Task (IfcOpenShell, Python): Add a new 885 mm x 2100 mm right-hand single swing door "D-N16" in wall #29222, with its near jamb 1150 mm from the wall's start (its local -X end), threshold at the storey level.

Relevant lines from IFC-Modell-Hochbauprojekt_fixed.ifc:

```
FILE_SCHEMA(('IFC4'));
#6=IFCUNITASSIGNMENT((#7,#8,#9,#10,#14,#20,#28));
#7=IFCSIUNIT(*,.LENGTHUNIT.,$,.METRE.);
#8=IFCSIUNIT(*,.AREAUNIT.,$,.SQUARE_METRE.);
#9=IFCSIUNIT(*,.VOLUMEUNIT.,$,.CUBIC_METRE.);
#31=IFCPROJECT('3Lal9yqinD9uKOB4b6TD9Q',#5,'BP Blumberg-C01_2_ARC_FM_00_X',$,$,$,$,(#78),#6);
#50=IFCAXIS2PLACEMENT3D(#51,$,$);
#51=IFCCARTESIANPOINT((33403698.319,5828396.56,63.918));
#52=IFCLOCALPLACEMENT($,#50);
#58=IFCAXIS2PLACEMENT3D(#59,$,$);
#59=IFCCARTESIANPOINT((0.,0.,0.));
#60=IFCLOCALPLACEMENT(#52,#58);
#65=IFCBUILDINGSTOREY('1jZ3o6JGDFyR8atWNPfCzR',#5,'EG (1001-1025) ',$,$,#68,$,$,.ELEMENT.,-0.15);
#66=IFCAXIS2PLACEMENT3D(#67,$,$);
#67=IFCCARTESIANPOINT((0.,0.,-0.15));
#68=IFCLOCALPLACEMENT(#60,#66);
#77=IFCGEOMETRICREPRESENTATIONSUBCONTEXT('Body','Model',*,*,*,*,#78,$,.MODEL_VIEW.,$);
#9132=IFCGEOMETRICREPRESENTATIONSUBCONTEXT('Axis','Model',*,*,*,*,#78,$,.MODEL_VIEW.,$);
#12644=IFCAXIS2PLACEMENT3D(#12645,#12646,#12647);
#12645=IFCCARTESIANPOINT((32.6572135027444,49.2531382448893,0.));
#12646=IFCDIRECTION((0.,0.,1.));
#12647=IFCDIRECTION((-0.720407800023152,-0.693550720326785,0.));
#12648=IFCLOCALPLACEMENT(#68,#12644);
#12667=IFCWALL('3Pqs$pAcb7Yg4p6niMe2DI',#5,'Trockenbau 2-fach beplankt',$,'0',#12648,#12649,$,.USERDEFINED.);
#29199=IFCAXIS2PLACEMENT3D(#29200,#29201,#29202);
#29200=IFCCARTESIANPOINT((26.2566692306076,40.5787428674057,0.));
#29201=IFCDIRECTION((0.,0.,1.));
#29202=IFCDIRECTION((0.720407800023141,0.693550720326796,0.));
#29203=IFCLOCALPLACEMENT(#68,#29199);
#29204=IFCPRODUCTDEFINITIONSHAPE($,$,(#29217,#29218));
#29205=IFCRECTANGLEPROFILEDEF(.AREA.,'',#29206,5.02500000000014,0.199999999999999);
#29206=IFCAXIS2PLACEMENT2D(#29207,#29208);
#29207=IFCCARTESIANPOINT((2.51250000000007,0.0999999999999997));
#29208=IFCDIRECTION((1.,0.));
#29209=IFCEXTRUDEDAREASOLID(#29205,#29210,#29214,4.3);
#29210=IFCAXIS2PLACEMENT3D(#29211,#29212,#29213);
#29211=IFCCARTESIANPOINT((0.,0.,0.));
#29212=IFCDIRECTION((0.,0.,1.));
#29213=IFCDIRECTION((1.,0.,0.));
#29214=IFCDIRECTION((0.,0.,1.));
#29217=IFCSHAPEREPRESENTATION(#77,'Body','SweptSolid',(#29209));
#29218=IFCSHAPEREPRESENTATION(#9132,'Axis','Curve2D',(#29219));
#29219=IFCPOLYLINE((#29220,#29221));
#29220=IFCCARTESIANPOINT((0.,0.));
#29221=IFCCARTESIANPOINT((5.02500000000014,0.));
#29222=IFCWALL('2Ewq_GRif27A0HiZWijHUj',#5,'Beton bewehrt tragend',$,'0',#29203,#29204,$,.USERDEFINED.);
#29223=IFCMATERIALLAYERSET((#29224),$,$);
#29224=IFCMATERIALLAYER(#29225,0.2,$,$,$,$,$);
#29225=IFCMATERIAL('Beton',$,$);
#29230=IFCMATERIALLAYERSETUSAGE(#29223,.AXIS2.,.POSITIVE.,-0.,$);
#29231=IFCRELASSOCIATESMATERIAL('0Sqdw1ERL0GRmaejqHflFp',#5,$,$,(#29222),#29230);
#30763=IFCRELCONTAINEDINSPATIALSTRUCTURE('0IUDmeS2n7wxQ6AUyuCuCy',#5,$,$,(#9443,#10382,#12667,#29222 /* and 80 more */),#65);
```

```python
import numpy as np
import ifcopenshell
import ifcopenshell.api.feature
import ifcopenshell.api.geometry
import ifcopenshell.api.root
import ifcopenshell.api.spatial
import ifcopenshell.geom
import ifcopenshell.util.element
import ifcopenshell.util.placement
import ifcopenshell.util.representation
import ifcopenshell.util.shape
import ifcopenshell.util.unit

model = ifcopenshell.open("IFC-Modell-Hochbauprojekt_fixed.ifc")
unit_scale = ifcopenshell.util.unit.calculate_unit_scale(model)
settings = ifcopenshell.geom.settings()


def volume(element):
    """Net volume in cubic metres, openings subtracted."""
    shape = ifcopenshell.geom.create_shape(settings, element)
    return ifcopenshell.util.shape.get_volume(shape.geometry)


wall = model.by_id(29222)
storey = ifcopenshell.util.element.get_container(wall, ifc_class="IfcBuildingStorey")
context = ifcopenshell.util.representation.get_context(model, "Model", "Body", "MODEL_VIEW")
before = volume(wall)

width, height, from_end, sill = 0.885, 2.1, 1.15, 0.0  # metres

# The wall runs along its own X axis, and the end named is its -X end.
wall_shape = ifcopenshell.geom.create_shape(settings, wall)
x, y, z = ifcopenshell.util.shape.get_vertices(wall_shape.geometry).T
start = x.min() + from_end
face, thickness = float(y.min()), float(y.max() - y.min())
wall_matrix = ifcopenshell.util.placement.get_local_placement(wall.ObjectPlacement)
level = ifcopenshell.util.placement.get_local_placement(storey.ObjectPlacement)[2, 3]


def in_wall(x, y):
    """Placement at x, y metres in the wall's axes, at sill height."""
    matrix = wall_matrix.copy()
    matrix[:, 3] = wall_matrix @ np.array([x / unit_scale, y / unit_scale, 0.0, 1.0])
    matrix[2, 3] = level + sill / unit_scale
    return matrix


# Opening: a box that overshoots both wall faces by 50 mm.
opening = ifcopenshell.api.root.create_entity(model, ifc_class="IfcOpeningElement", predefined_type="OPENING")
box = ifcopenshell.api.geometry.add_wall_representation(
    model, context=context, length=width, height=height, thickness=thickness + 0.1
)
ifcopenshell.api.geometry.assign_representation(model, product=opening, representation=box)
ifcopenshell.api.geometry.edit_object_placement(model, product=opening, matrix=in_wall(start, face - 0.05), is_si=False)
ifcopenshell.api.feature.add_feature(model, feature=opening, element=wall)

door = ifcopenshell.api.root.create_entity(model, ifc_class="IfcDoor", name="D-N16", predefined_type="DOOR")
door.OverallWidth, door.OverallHeight = width / unit_scale, height / unit_scale
door.OperationType = "SINGLE_SWING_RIGHT"
body = ifcopenshell.api.geometry.add_door_representation(
    model,
    context=context,
    overall_width=door.OverallWidth,
    overall_height=door.OverallHeight,
    operation_type="SINGLE_SWING_RIGHT",
    lining_properties={"LiningDepth": thickness / unit_scale, "ThresholdDepth": thickness / unit_scale},
)
ifcopenshell.api.geometry.assign_representation(model, product=door, representation=body)
ifcopenshell.api.spatial.assign_container(model, products=[door], relating_structure=storey)
ifcopenshell.api.feature.add_filling(model, opening=opening, element=door)

# The lining spans the wall, so the door starts at the wall face.
ifcopenshell.api.geometry.edit_object_placement(model, product=door, matrix=in_wall(start, face), is_si=False)

after = volume(wall)

print(f"wall volume {before:.3f} -> {after:.3f} m3")

model.write("IFC-Modell-Hochbauprojekt_fixed_edited.ifc")
```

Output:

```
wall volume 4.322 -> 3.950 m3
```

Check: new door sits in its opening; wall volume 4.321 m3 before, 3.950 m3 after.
